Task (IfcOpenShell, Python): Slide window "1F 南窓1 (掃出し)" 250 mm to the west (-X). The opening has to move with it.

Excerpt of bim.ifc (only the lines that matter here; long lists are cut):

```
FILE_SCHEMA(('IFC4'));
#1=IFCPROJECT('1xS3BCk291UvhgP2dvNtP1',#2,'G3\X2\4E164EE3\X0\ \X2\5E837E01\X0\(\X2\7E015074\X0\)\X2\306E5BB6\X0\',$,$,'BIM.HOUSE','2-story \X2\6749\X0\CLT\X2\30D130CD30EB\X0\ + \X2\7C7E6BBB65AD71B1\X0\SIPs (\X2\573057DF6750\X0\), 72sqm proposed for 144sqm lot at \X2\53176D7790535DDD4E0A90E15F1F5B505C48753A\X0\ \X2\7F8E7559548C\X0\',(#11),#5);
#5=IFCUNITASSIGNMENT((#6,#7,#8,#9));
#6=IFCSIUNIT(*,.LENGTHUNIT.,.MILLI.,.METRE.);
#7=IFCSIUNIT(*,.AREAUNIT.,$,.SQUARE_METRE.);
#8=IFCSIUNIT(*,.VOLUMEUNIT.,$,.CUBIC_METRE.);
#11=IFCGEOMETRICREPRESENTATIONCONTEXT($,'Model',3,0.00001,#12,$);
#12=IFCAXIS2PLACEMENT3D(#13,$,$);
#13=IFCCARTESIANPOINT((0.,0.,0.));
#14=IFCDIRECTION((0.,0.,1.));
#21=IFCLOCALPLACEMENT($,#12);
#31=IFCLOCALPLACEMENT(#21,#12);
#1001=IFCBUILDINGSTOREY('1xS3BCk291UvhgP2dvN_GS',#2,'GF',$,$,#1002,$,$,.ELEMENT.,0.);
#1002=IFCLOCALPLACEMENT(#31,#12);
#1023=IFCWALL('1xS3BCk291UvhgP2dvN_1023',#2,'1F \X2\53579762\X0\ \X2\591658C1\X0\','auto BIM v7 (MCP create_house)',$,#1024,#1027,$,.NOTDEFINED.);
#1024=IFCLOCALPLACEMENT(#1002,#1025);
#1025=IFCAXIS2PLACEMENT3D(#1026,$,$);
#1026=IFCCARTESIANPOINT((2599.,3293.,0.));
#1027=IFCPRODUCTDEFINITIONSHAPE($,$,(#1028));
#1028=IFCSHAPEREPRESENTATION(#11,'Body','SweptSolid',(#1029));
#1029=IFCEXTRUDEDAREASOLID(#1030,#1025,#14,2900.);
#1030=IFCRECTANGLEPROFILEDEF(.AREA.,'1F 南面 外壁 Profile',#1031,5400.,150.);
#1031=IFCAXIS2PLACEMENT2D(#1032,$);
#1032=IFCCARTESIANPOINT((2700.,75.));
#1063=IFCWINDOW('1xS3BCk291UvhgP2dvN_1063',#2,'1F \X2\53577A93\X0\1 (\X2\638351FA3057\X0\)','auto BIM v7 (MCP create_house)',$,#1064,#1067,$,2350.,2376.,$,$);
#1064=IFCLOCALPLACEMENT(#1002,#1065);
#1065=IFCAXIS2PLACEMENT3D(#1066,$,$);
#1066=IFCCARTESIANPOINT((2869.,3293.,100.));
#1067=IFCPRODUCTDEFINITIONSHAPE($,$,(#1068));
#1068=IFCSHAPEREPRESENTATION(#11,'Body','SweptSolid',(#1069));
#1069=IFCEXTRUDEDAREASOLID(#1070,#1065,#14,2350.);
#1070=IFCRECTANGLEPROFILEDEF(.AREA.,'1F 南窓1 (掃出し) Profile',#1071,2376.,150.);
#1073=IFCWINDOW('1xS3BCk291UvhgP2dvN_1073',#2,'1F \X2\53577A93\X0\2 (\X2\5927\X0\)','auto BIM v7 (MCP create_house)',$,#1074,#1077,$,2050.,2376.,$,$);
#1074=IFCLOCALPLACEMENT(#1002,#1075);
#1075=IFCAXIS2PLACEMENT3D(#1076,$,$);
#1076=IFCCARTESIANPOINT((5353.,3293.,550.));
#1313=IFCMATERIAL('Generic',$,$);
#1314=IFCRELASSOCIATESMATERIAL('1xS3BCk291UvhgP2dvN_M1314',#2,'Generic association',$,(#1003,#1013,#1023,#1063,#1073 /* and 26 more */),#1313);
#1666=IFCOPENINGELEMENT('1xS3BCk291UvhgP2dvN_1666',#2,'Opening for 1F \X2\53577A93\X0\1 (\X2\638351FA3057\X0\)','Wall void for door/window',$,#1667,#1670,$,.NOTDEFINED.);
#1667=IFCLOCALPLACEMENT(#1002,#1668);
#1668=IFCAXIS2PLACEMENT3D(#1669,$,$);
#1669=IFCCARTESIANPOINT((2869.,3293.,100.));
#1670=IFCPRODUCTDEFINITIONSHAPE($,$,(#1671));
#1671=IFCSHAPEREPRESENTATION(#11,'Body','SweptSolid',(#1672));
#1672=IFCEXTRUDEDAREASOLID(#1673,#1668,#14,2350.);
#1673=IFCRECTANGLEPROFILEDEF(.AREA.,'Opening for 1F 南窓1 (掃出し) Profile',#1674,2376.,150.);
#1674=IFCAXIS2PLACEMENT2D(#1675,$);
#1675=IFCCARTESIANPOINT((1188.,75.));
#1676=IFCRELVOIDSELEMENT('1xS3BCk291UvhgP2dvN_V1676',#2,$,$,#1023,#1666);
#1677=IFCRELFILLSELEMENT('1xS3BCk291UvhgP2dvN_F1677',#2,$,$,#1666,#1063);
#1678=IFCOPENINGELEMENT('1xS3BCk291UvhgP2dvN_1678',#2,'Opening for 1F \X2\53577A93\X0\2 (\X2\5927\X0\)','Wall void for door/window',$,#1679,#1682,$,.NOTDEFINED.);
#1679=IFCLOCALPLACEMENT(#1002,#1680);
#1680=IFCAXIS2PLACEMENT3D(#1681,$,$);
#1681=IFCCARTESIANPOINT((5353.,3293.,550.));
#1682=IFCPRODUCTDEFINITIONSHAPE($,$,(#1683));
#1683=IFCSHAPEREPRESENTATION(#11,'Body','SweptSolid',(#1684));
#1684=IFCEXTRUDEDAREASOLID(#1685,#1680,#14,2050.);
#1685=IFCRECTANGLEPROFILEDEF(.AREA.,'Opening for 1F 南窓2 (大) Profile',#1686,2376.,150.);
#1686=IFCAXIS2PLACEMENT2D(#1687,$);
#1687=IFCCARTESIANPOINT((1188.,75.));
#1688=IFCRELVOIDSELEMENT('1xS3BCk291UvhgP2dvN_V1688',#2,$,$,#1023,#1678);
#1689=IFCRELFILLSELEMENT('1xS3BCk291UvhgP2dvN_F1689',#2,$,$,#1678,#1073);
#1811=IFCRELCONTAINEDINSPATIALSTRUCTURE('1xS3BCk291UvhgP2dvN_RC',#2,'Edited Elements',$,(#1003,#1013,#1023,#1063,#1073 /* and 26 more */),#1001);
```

```python
import ifcopenshell
import ifcopenshell.api.geometry
import ifcopenshell.util.placement

model = ifcopenshell.open("bim.ifc")

window = model.by_guid("1xS3BCk291UvhgP2dvN_1063")
opening = window.FillsVoids[0].RelatingOpeningElement
wall = opening.VoidsElements[0].RelatingBuildingElement

wall_matrix = ifcopenshell.util.placement.get_local_placement(wall.ObjectPlacement)
shift = wall_matrix[:3, 0] * -250.0
before = ifcopenshell.util.placement.get_local_placement(window.ObjectPlacement)[:3, 3].copy()

# The window is not placed relative to its opening, so move both.
for product in (opening, window):
    matrix = ifcopenshell.util.placement.get_local_placement(product.ObjectPlacement)
    matrix[:3, 3] += shift
    ifcopenshell.api.geometry.edit_object_placement(model, product=product, matrix=matrix, is_si=False)

after = ifcopenshell.util.placement.get_local_placement(window.ObjectPlacement)[:3, 3]
print("window moved by", (after - before).round(3) + 0.0)

model.write("bim-out.ifc")
```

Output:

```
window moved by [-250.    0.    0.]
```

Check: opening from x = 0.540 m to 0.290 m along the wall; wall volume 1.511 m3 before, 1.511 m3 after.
